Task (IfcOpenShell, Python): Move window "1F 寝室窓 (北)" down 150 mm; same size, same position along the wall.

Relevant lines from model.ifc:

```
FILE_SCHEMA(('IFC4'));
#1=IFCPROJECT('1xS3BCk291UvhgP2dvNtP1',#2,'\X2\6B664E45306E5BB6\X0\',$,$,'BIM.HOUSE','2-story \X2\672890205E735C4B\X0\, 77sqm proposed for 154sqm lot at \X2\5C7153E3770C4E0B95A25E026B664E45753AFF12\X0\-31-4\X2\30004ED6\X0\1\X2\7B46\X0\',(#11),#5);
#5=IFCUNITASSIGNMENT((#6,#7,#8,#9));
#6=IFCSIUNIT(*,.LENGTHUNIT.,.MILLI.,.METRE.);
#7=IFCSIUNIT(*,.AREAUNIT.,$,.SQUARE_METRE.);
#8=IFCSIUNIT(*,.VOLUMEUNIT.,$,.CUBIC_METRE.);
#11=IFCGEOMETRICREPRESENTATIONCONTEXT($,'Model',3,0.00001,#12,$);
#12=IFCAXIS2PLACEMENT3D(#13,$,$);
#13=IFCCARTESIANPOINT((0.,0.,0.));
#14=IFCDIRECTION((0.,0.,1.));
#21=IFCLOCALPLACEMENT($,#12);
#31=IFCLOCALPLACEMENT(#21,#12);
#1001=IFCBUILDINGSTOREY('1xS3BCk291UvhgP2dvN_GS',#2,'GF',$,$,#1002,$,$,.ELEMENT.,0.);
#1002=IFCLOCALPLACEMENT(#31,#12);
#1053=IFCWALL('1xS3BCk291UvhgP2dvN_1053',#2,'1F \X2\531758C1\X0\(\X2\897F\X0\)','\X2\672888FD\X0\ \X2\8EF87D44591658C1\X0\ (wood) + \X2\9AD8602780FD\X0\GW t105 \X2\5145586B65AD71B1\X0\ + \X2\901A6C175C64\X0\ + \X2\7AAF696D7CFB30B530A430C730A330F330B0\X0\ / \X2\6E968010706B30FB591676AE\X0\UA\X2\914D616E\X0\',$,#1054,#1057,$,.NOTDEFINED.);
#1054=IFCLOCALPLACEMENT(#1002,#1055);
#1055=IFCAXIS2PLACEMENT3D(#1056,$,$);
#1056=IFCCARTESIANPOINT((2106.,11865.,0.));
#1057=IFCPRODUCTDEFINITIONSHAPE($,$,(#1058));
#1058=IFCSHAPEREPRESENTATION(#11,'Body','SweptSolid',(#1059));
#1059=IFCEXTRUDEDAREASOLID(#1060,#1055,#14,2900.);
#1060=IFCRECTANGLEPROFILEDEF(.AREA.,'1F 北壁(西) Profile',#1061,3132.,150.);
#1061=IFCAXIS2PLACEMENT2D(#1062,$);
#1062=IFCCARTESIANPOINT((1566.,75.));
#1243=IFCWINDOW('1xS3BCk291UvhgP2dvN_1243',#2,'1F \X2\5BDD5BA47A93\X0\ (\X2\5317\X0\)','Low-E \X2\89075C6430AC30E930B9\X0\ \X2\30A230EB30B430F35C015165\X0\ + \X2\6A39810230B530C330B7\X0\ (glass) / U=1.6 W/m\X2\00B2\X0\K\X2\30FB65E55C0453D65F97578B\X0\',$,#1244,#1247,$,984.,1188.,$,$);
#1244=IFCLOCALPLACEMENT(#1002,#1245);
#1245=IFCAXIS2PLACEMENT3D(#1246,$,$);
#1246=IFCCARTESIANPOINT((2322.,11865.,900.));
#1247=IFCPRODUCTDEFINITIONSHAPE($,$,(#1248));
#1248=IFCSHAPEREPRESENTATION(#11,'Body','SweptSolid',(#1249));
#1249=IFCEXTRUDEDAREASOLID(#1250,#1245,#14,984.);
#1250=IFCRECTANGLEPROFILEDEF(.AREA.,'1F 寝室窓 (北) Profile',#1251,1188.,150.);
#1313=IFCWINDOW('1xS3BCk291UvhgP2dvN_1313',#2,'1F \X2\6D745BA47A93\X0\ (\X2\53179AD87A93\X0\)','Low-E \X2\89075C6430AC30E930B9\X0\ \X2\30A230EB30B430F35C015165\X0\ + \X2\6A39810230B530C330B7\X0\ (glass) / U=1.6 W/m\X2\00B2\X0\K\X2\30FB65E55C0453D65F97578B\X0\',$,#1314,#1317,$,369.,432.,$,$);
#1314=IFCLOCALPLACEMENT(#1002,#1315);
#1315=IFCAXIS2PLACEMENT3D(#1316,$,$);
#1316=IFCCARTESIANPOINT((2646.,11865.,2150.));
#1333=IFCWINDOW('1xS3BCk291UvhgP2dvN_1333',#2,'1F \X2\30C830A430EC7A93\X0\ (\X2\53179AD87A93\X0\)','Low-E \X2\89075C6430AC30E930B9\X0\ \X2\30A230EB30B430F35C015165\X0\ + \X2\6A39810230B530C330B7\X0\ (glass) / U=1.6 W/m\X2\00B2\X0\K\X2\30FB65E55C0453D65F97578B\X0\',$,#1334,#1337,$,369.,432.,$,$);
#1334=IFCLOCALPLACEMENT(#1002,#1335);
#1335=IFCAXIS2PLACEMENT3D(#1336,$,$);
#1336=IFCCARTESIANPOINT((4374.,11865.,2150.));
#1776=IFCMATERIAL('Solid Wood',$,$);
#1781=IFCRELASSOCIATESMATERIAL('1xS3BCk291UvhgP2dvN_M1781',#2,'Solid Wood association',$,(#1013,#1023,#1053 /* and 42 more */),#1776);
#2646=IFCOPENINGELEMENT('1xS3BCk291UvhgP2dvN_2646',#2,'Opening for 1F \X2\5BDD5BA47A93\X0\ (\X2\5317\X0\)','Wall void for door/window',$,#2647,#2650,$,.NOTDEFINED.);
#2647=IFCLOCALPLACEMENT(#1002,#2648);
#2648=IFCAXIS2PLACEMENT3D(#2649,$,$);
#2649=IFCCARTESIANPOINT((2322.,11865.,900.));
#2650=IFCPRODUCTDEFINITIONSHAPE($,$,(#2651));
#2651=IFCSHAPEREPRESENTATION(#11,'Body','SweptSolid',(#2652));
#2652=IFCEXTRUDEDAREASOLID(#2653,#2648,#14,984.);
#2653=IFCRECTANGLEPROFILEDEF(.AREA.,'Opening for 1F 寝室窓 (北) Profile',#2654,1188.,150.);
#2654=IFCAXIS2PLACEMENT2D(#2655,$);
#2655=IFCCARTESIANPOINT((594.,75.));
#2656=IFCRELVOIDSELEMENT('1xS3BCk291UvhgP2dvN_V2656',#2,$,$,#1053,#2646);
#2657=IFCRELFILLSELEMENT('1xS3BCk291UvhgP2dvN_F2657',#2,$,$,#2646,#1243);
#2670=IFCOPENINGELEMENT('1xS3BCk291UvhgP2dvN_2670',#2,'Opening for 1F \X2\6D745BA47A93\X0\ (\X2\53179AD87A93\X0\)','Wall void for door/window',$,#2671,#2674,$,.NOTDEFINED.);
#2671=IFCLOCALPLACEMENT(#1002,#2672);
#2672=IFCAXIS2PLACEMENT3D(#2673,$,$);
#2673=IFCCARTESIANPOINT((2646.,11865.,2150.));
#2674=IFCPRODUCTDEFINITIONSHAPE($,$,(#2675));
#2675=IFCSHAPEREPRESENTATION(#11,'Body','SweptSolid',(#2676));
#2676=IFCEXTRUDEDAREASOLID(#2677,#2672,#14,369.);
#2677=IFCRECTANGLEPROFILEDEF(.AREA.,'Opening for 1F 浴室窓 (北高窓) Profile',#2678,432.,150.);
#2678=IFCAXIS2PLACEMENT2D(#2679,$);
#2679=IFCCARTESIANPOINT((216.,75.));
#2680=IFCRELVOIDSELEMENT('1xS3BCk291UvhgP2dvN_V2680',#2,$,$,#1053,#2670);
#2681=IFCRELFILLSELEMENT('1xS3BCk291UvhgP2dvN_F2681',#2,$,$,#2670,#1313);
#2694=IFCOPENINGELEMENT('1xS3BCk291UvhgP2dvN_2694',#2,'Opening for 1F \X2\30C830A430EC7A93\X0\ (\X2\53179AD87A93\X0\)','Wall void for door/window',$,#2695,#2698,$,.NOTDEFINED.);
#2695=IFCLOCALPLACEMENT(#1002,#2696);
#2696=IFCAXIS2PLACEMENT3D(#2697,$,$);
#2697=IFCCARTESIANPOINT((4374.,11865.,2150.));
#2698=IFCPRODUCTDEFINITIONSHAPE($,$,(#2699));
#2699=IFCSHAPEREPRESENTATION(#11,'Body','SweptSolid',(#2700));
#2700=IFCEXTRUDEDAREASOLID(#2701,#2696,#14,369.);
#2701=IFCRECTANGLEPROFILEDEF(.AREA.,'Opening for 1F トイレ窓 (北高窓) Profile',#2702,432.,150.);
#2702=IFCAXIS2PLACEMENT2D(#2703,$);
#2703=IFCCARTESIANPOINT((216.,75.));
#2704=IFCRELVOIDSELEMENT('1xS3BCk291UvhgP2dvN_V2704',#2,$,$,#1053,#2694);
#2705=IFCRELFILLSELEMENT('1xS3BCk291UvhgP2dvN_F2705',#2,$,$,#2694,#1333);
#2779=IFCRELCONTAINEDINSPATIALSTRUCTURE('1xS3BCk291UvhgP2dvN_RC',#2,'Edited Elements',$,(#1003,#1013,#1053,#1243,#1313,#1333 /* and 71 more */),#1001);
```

```python
import numpy as np
import ifcopenshell
import ifcopenshell.api.geometry
import ifcopenshell.util.placement
import ifcopenshell.util.unit

model = ifcopenshell.open("model.ifc")
unit_scale = ifcopenshell.util.unit.calculate_unit_scale(model)

window = model.by_guid("1xS3BCk291UvhgP2dvN_1243")
opening = window.FillsVoids[0].RelatingOpeningElement
dz = -150.0

shift = np.array([0.0, 0.0, dz])
# The window is not placed relative to its opening, so move both.
for product in (opening, window):
    matrix = ifcopenshell.util.placement.get_local_placement(product.ObjectPlacement)
    matrix[:3, 3] += shift
    ifcopenshell.api.geometry.edit_object_placement(model, product=product, matrix=matrix, is_si=False)

print(f"moved by {dz * unit_scale:+.3f} m")

model.write("model_rev.ifc")
```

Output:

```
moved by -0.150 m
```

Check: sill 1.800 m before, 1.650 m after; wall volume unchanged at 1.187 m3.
